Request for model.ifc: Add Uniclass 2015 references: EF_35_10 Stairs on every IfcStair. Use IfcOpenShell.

First a look at what the model holds.

```python
import ifcopenshell

model = ifcopenshell.open("model.ifc")
print(model.schema)
print("classifications:", [c.Name for c in model.by_type("IfcClassification")])
for ifc_class in ("IfcDoor", "IfcRoof", "IfcStair", "IfcWall", "IfcWindow"):
    print(ifc_class, len(model.by_type(ifc_class)))
```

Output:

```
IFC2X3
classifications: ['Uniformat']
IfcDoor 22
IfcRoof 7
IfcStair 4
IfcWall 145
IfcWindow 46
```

```python
import ifcopenshell
import ifcopenshell.api.classification

model = ifcopenshell.open("model.ifc")

# IFC2X3 requires Source and Edition and has no link from the project to the system.
system = model.create_entity("IfcClassification", Source="NBS", Edition="2015", Name="Uniclass 2015")

codes = {
    "IfcStair": ("EF_35_10", "Stairs"),
}
for ifc_class, (code, name) in codes.items():
    products = model.by_type(ifc_class)
    ifcopenshell.api.classification.add_reference(
        model, products=products, classification=system, identification=code, name=name
    )
    print(code, len(products))

model.write("model_v2.ifc")
```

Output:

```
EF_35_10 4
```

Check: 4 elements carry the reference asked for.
